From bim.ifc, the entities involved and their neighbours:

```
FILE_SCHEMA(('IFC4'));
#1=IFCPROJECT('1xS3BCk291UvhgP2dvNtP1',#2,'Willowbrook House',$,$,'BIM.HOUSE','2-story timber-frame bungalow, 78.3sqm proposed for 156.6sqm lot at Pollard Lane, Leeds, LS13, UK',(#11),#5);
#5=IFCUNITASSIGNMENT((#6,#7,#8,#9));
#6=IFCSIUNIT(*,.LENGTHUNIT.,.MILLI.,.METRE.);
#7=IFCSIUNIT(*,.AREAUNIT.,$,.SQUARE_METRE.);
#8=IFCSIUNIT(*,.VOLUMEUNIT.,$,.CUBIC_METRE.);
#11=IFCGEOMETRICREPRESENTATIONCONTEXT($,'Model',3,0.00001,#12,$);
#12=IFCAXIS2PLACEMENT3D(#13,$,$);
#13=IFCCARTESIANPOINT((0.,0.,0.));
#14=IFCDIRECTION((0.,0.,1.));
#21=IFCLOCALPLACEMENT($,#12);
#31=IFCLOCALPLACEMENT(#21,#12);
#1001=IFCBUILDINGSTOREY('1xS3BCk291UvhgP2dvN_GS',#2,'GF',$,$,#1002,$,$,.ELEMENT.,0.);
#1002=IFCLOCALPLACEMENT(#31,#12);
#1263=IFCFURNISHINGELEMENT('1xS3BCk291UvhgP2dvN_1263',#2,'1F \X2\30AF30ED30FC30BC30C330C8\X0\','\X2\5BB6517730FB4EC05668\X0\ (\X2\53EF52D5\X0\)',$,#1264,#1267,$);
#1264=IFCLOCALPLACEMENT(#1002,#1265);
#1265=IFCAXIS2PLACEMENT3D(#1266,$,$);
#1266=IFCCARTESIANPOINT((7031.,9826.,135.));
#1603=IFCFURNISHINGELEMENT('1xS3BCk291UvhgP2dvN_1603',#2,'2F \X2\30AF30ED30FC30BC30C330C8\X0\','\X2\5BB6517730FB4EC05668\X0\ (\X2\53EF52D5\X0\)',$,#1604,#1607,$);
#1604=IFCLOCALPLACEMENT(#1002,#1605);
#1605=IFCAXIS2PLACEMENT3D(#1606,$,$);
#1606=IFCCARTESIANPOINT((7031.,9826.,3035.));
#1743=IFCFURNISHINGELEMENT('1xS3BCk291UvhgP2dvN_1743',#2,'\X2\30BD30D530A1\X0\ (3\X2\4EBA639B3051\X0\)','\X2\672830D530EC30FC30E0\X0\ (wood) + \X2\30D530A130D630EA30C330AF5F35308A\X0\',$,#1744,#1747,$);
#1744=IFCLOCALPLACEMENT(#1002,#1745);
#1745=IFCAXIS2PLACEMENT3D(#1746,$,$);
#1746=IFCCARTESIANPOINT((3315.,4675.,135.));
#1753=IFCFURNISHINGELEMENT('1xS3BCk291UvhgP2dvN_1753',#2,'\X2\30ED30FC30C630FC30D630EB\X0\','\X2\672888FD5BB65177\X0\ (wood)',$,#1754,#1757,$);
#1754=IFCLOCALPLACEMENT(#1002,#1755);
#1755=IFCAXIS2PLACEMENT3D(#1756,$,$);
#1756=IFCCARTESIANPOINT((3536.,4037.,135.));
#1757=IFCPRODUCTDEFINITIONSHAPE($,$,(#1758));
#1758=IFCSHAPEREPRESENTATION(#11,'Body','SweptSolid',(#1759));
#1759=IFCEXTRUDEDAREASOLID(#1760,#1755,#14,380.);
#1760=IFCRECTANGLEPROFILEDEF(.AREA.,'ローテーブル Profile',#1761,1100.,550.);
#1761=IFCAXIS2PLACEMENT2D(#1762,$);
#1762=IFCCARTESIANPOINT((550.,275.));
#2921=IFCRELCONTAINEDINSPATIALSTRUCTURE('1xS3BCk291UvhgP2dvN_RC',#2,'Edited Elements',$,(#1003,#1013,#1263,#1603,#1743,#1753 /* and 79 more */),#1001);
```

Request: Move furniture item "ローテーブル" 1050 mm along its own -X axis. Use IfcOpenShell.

```python
import ifcopenshell
import ifcopenshell.api.geometry
import ifcopenshell.util.placement

model = ifcopenshell.open("bim.ifc")

item = model.by_id(1753)
matrix = ifcopenshell.util.placement.get_local_placement(item.ObjectPlacement)
matrix[:3, 3] -= matrix[:3, 0] * 1050.0
ifcopenshell.api.geometry.edit_object_placement(model, product=item, matrix=matrix, is_si=False)

print(ifcopenshell.util.placement.get_local_placement(item.ObjectPlacement).round(3) + 0.0)

model.write("bim_v2.ifc")
```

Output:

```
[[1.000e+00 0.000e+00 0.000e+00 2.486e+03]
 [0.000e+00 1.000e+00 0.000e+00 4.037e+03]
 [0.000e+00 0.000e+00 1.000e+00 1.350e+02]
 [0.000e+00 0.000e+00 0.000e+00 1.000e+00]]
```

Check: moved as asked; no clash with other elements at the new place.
